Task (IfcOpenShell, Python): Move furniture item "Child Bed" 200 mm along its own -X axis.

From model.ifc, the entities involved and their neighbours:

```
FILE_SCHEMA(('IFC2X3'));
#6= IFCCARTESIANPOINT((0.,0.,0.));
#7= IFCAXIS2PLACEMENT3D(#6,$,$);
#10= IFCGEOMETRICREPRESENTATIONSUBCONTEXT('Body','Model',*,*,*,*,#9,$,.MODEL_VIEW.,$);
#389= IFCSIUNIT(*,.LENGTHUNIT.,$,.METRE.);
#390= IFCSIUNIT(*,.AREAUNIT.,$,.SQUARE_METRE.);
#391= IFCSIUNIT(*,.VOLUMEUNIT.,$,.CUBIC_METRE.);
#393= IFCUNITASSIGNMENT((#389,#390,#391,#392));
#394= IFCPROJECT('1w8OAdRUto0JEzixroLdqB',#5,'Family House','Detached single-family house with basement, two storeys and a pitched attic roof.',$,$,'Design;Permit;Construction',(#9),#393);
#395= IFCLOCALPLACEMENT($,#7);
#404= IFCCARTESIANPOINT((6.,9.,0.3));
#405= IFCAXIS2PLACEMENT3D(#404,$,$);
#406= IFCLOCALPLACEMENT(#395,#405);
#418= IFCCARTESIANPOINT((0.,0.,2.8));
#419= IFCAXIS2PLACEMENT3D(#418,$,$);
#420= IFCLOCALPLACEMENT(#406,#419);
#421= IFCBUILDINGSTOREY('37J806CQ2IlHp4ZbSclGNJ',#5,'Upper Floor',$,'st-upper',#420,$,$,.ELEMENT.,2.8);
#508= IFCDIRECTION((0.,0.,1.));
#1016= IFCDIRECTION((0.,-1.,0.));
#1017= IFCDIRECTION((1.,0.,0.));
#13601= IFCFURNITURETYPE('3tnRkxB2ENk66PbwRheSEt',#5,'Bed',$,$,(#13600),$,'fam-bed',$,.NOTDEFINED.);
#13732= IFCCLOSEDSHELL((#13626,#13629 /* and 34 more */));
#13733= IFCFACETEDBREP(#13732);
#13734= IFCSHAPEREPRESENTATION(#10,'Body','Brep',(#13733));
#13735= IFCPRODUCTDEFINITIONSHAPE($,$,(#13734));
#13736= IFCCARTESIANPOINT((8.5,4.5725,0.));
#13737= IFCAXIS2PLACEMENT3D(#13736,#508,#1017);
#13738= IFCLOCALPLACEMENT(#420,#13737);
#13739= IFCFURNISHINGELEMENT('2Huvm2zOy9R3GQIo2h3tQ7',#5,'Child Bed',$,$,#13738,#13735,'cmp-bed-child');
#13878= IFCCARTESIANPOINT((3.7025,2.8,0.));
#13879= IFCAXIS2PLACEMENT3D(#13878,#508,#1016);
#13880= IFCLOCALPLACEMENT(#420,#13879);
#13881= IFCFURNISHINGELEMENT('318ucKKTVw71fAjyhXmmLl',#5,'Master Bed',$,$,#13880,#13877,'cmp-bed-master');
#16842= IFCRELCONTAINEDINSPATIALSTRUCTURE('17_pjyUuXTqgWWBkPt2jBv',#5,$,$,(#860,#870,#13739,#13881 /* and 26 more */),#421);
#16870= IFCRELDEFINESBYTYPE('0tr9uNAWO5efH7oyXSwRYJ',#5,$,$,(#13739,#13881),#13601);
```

```python
import ifcopenshell
import ifcopenshell.api.geometry
import ifcopenshell.util.placement
import ifcopenshell.util.unit

model = ifcopenshell.open("model.ifc")
unit_scale = ifcopenshell.util.unit.calculate_unit_scale(model)

item = model.by_guid("2Huvm2zOy9R3GQIo2h3tQ7")
matrix = ifcopenshell.util.placement.get_local_placement(item.ObjectPlacement)
matrix[:3, 3] -= matrix[:3, 0] * 0.2 / unit_scale
ifcopenshell.api.geometry.edit_object_placement(model, product=item, matrix=matrix, is_si=False)

print(ifcopenshell.util.placement.get_local_placement(item.ObjectPlacement).round(3) + 0.0)

model.write("model_rev.ifc")
```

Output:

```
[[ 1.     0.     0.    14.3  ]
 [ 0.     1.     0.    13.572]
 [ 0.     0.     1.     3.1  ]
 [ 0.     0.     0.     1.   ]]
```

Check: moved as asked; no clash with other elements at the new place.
